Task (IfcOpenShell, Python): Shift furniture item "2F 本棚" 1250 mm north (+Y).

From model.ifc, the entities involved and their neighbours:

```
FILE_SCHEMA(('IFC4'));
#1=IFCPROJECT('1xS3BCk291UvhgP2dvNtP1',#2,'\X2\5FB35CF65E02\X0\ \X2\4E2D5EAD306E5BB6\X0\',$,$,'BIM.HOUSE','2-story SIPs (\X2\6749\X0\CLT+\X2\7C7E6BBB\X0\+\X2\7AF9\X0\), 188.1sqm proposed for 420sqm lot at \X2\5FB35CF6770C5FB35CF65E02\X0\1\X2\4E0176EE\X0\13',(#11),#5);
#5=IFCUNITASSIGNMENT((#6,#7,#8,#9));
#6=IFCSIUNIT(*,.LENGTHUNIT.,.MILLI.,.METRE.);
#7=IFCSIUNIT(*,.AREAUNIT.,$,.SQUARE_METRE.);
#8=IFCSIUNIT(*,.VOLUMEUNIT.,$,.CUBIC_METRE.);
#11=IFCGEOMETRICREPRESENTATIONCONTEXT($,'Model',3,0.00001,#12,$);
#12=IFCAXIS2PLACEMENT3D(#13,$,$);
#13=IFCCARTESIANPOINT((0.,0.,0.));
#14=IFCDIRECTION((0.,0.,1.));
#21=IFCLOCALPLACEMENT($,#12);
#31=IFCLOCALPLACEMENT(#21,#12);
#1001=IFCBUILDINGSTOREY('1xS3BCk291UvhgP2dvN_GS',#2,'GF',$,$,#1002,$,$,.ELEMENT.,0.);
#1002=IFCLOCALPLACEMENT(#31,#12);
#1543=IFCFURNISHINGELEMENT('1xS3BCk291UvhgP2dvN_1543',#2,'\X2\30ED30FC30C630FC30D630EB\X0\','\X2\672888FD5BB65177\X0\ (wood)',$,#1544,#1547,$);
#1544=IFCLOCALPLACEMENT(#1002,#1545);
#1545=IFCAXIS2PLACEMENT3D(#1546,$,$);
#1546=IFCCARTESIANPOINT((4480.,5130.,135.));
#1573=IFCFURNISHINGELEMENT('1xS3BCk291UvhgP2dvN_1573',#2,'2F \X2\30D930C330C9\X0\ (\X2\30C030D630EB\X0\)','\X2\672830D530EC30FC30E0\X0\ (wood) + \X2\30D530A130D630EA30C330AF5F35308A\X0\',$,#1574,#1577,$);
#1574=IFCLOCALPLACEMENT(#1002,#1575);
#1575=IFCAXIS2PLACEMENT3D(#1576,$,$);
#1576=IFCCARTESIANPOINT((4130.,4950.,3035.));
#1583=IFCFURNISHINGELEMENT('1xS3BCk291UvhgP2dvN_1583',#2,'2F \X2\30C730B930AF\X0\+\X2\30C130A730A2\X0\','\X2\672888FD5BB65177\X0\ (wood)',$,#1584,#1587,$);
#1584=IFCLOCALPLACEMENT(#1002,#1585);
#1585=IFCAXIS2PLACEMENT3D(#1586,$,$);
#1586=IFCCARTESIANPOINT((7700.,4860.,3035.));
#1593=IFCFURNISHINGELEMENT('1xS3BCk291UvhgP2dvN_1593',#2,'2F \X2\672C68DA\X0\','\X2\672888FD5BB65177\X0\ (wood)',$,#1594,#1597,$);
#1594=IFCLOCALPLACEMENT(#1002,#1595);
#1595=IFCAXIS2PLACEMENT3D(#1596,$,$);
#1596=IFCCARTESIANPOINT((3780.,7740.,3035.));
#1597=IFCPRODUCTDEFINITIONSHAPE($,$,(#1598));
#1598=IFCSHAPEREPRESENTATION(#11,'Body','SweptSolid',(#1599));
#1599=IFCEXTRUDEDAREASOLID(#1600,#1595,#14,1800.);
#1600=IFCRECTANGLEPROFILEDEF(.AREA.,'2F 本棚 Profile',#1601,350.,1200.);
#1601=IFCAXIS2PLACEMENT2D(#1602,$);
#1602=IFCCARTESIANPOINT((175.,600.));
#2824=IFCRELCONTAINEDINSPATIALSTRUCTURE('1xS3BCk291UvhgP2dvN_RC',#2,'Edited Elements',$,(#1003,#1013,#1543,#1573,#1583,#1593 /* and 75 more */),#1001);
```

```python
import ifcopenshell
import ifcopenshell.api.geometry
import ifcopenshell.util.placement
import ifcopenshell.util.unit

model = ifcopenshell.open("model.ifc")
unit_scale = ifcopenshell.util.unit.calculate_unit_scale(model)

item = model.by_guid("1xS3BCk291UvhgP2dvN_1593")
matrix = ifcopenshell.util.placement.get_local_placement(item.ObjectPlacement)
matrix[1, 3] += 1.25 / unit_scale
ifcopenshell.api.geometry.edit_object_placement(model, product=item, matrix=matrix, is_si=False)

print(ifcopenshell.util.placement.get_local_placement(item.ObjectPlacement).round(3) + 0.0)

model.write("model-out.ifc")
```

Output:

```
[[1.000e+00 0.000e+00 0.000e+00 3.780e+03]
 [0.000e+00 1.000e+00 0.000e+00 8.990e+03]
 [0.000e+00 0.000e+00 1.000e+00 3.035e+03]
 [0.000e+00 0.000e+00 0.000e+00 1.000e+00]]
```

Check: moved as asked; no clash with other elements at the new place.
